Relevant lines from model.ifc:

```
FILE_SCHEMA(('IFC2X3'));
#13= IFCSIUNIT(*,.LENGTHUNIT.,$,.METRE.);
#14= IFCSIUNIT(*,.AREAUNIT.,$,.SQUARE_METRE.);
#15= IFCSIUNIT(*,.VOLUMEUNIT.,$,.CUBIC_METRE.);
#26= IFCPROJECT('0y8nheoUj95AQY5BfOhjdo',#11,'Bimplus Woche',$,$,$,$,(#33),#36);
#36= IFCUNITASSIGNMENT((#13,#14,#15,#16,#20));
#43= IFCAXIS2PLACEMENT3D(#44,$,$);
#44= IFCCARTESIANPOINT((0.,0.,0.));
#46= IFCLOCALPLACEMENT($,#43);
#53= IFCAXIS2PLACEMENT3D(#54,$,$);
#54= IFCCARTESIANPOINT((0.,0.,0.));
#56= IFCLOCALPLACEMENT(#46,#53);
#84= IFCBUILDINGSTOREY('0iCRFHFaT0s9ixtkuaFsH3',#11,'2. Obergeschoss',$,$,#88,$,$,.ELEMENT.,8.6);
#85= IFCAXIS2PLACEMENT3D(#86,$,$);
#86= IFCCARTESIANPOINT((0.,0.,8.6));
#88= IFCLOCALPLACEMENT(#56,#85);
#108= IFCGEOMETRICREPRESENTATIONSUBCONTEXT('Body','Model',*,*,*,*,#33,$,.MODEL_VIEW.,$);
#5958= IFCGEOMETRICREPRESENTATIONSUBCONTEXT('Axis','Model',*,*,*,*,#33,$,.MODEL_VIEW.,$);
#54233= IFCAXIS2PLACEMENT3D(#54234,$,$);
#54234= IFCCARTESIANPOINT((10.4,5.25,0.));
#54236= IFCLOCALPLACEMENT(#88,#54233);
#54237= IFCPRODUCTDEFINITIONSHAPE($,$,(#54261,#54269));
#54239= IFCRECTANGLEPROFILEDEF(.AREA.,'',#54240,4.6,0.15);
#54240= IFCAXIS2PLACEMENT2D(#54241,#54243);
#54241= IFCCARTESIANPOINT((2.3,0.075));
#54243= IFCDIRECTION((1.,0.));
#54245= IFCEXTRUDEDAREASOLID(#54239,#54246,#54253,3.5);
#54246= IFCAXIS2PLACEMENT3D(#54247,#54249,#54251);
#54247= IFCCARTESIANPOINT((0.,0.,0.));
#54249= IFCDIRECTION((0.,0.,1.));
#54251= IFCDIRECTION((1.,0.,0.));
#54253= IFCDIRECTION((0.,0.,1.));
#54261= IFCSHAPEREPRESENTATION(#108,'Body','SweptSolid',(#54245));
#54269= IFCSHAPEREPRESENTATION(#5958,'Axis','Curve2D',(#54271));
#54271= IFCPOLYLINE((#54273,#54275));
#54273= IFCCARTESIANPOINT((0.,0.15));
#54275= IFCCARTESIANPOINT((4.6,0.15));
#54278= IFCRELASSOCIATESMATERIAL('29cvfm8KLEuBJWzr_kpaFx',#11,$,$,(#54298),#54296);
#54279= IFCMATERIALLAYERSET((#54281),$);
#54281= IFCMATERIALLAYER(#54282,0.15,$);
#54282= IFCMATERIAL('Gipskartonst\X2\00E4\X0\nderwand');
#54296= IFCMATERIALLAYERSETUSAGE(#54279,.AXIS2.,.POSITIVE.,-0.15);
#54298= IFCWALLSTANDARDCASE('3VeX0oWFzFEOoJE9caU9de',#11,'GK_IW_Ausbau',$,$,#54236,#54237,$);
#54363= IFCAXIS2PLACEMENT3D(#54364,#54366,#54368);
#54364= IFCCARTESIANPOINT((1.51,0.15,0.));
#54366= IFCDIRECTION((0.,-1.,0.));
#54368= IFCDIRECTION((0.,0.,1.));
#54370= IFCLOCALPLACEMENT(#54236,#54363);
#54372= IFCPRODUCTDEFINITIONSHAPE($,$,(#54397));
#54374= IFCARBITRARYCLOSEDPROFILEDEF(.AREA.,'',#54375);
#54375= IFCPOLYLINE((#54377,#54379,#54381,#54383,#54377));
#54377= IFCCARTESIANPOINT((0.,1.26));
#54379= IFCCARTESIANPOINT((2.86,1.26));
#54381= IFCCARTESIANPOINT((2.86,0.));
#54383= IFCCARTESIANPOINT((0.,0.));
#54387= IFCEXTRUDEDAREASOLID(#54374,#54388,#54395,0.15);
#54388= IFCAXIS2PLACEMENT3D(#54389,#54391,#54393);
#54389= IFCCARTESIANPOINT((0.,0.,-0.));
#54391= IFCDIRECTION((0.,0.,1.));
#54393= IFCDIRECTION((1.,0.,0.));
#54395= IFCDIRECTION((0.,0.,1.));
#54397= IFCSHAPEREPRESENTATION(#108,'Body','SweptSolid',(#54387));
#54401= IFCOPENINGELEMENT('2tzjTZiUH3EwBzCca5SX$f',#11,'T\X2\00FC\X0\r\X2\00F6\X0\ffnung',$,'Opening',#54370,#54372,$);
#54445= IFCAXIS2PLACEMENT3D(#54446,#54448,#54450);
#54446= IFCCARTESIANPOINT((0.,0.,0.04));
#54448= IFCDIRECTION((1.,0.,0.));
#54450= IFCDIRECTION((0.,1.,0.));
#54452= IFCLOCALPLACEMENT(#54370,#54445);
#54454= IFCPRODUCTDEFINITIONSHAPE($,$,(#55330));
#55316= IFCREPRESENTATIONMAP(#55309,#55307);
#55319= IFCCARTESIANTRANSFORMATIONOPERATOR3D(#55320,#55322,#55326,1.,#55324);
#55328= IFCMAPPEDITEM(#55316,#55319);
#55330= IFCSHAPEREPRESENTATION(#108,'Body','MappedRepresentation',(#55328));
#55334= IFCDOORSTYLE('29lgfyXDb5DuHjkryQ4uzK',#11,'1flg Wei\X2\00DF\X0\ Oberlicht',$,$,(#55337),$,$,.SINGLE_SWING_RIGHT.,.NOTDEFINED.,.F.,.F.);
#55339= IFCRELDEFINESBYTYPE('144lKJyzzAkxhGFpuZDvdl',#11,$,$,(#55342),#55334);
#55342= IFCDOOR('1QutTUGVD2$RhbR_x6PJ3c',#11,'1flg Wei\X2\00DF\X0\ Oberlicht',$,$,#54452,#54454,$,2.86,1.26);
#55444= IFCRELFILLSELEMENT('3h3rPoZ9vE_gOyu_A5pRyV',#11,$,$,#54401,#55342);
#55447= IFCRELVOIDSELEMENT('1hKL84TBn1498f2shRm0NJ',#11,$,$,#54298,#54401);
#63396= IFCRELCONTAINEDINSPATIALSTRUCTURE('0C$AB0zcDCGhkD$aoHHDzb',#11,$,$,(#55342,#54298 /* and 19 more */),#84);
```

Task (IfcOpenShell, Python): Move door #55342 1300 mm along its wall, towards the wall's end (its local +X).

```python
import ifcopenshell
import ifcopenshell.api.geometry
import ifcopenshell.util.placement

model = ifcopenshell.open("model.ifc")

door = model.by_guid("1QutTUGVD2$RhbR_x6PJ3c")
opening = door.FillsVoids[0].RelatingOpeningElement
wall = opening.VoidsElements[0].RelatingBuildingElement

wall_matrix = ifcopenshell.util.placement.get_local_placement(wall.ObjectPlacement)
shift = wall_matrix[:3, 0] * 1.3
before = ifcopenshell.util.placement.get_local_placement(door.ObjectPlacement)[:3, 3].copy()

# The door is placed relative to its opening, so it follows when the opening moves.
matrix = ifcopenshell.util.placement.get_local_placement(opening.ObjectPlacement)
matrix[:3, 3] += shift
ifcopenshell.api.geometry.edit_object_placement(
    model, product=opening, matrix=matrix, is_si=False, should_transform_children=True
)

after = ifcopenshell.util.placement.get_local_placement(door.ObjectPlacement)[:3, 3]
print("door moved by", (after - before).round(3) + 0.0)

model.write("model_edited.ifc")
```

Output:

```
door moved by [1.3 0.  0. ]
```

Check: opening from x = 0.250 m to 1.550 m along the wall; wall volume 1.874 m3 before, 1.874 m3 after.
